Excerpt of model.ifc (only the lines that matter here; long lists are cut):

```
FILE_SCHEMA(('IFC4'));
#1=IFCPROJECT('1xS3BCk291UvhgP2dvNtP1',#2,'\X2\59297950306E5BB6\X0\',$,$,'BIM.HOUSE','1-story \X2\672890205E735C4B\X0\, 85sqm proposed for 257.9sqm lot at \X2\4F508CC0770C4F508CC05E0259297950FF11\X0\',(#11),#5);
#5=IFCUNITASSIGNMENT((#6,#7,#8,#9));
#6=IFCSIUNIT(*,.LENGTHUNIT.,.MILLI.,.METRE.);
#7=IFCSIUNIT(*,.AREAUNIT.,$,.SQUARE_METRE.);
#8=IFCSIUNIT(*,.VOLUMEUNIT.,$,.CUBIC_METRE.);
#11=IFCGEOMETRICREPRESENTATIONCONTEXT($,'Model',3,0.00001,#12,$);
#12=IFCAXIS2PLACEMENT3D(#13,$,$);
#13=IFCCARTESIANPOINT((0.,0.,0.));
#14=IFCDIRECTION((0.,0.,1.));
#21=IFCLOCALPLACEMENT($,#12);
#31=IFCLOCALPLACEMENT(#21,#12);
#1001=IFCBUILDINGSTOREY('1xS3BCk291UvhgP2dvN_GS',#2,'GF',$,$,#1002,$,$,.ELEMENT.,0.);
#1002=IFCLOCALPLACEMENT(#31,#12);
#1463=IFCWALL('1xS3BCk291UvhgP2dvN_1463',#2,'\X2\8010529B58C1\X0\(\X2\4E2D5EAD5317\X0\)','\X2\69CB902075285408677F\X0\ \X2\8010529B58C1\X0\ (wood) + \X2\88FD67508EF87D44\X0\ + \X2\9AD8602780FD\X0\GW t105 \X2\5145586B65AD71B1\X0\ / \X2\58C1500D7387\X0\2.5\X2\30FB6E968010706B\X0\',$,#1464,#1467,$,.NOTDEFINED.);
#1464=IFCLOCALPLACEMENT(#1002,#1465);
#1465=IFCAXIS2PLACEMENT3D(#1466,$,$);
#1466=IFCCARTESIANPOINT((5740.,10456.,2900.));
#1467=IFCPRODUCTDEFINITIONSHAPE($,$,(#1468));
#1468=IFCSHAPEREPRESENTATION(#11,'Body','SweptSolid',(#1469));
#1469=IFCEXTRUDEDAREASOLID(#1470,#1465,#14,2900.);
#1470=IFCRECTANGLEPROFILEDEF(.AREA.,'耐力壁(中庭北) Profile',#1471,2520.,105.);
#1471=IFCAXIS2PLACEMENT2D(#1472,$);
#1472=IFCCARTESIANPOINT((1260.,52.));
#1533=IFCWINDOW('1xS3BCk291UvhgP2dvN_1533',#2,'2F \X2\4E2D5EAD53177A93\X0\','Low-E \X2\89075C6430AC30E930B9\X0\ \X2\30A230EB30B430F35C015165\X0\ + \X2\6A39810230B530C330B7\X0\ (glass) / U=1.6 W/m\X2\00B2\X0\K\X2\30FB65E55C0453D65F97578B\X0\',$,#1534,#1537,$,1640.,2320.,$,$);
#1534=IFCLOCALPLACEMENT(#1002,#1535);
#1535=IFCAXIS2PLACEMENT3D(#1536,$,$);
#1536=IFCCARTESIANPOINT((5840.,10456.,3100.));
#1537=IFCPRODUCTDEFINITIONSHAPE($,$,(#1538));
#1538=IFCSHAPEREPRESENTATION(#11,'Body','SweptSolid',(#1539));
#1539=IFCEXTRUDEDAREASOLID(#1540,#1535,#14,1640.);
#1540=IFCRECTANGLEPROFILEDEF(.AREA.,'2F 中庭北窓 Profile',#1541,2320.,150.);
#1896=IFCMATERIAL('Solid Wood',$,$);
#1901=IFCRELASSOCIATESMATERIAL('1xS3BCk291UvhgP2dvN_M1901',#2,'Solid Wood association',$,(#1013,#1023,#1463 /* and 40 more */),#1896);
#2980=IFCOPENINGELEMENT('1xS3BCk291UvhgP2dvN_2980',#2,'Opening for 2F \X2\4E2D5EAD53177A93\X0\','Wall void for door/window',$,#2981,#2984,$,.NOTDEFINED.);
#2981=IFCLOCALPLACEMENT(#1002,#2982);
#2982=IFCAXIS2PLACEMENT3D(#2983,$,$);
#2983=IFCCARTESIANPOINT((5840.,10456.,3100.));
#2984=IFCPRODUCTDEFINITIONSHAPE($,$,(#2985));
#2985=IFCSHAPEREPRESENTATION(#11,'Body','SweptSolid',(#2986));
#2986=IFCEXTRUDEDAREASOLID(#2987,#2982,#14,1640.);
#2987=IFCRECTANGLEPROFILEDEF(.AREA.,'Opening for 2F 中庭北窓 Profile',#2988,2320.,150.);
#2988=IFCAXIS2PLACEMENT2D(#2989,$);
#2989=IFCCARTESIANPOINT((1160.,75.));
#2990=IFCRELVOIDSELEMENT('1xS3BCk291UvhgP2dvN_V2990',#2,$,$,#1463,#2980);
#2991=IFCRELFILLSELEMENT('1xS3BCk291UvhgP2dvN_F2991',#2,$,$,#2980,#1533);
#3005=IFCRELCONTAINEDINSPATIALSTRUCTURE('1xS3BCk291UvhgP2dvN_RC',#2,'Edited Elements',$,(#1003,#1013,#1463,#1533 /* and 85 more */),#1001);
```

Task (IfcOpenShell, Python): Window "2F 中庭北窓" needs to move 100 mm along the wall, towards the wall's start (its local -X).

```python
import ifcopenshell
import ifcopenshell.api.geometry
import ifcopenshell.util.placement
import ifcopenshell.util.unit

model = ifcopenshell.open("model.ifc")
unit_scale = ifcopenshell.util.unit.calculate_unit_scale(model)

window = model.by_guid("1xS3BCk291UvhgP2dvN_1533")
opening = window.FillsVoids[0].RelatingOpeningElement
wall = opening.VoidsElements[0].RelatingBuildingElement

wall_matrix = ifcopenshell.util.placement.get_local_placement(wall.ObjectPlacement)
shift = wall_matrix[:3, 0] * -0.1 / unit_scale
before = ifcopenshell.util.placement.get_local_placement(window.ObjectPlacement)[:3, 3].copy()

# The window is not placed relative to its opening, so move both.
for product in (opening, window):
    matrix = ifcopenshell.util.placement.get_local_placement(product.ObjectPlacement)
    matrix[:3, 3] += shift
    ifcopenshell.api.geometry.edit_object_placement(model, product=product, matrix=matrix, is_si=False)

after = ifcopenshell.util.placement.get_local_placement(window.ObjectPlacement)[:3, 3]
print("window moved by", (after - before).round(3) + 0.0)

model.write("model-out.ifc")
```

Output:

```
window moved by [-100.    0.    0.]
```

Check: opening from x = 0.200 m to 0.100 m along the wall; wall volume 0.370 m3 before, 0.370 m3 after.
